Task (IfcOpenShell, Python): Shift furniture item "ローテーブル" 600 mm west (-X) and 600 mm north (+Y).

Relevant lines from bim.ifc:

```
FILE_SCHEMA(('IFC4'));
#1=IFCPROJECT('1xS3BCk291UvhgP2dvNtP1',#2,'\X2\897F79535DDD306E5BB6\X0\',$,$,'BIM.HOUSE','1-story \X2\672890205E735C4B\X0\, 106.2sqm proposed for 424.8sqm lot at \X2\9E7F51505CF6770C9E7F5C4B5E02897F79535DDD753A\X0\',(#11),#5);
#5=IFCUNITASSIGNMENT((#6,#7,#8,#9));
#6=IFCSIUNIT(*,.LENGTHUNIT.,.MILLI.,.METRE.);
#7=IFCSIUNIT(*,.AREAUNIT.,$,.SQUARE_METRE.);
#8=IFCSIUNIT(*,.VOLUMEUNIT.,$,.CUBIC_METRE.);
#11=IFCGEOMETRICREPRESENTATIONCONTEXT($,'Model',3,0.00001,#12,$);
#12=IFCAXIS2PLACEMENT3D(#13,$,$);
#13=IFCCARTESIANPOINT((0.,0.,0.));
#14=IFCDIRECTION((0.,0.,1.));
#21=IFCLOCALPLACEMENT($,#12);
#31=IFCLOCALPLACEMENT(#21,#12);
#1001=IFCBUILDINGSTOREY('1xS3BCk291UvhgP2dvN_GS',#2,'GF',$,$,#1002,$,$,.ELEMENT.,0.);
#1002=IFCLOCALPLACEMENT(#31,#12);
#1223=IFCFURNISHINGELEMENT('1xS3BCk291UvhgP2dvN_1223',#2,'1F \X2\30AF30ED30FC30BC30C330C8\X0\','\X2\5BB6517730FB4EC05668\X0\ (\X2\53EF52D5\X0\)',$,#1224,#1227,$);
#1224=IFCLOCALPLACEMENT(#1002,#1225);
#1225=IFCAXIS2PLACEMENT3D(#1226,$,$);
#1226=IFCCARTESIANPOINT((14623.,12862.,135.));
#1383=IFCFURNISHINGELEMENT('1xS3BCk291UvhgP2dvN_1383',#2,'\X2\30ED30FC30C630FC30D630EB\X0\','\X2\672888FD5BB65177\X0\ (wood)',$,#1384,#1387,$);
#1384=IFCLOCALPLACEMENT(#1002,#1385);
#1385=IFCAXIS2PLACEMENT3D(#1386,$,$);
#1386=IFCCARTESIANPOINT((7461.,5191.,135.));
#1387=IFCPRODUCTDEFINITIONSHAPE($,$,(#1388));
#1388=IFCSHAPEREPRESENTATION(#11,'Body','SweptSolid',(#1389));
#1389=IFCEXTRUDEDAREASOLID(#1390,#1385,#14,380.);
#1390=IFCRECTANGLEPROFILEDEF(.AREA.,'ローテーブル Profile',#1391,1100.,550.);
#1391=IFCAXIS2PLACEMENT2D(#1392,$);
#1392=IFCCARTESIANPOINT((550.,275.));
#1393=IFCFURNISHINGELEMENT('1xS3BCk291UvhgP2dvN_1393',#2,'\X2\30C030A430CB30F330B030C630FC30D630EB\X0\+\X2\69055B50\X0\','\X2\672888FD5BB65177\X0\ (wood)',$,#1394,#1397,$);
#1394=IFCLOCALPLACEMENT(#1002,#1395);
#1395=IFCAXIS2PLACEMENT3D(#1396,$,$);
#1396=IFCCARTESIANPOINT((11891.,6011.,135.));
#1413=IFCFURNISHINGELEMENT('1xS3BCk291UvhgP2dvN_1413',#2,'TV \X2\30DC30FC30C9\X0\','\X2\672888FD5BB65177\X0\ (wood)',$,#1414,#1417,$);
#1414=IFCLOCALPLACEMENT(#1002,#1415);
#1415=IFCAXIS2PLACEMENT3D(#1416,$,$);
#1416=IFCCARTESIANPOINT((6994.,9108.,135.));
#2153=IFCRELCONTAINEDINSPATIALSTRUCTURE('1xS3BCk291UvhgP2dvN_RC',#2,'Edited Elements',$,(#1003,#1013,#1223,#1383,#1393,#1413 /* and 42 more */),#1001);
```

```python
import ifcopenshell
import ifcopenshell.api.geometry
import ifcopenshell.util.placement
import ifcopenshell.util.unit

model = ifcopenshell.open("bim.ifc")
unit_scale = ifcopenshell.util.unit.calculate_unit_scale(model)

item = model.by_id(1383)
matrix = ifcopenshell.util.placement.get_local_placement(item.ObjectPlacement)
matrix[0, 3] -= 0.6 / unit_scale
matrix[1, 3] += 0.6 / unit_scale
ifcopenshell.api.geometry.edit_object_placement(model, product=item, matrix=matrix, is_si=False)

print(ifcopenshell.util.placement.get_local_placement(item.ObjectPlacement).round(3) + 0.0)

model.write("bim_v2.ifc")
```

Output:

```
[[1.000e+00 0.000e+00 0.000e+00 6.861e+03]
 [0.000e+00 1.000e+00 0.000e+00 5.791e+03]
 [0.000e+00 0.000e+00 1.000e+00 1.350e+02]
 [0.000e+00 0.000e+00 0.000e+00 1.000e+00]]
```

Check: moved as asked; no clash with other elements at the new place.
